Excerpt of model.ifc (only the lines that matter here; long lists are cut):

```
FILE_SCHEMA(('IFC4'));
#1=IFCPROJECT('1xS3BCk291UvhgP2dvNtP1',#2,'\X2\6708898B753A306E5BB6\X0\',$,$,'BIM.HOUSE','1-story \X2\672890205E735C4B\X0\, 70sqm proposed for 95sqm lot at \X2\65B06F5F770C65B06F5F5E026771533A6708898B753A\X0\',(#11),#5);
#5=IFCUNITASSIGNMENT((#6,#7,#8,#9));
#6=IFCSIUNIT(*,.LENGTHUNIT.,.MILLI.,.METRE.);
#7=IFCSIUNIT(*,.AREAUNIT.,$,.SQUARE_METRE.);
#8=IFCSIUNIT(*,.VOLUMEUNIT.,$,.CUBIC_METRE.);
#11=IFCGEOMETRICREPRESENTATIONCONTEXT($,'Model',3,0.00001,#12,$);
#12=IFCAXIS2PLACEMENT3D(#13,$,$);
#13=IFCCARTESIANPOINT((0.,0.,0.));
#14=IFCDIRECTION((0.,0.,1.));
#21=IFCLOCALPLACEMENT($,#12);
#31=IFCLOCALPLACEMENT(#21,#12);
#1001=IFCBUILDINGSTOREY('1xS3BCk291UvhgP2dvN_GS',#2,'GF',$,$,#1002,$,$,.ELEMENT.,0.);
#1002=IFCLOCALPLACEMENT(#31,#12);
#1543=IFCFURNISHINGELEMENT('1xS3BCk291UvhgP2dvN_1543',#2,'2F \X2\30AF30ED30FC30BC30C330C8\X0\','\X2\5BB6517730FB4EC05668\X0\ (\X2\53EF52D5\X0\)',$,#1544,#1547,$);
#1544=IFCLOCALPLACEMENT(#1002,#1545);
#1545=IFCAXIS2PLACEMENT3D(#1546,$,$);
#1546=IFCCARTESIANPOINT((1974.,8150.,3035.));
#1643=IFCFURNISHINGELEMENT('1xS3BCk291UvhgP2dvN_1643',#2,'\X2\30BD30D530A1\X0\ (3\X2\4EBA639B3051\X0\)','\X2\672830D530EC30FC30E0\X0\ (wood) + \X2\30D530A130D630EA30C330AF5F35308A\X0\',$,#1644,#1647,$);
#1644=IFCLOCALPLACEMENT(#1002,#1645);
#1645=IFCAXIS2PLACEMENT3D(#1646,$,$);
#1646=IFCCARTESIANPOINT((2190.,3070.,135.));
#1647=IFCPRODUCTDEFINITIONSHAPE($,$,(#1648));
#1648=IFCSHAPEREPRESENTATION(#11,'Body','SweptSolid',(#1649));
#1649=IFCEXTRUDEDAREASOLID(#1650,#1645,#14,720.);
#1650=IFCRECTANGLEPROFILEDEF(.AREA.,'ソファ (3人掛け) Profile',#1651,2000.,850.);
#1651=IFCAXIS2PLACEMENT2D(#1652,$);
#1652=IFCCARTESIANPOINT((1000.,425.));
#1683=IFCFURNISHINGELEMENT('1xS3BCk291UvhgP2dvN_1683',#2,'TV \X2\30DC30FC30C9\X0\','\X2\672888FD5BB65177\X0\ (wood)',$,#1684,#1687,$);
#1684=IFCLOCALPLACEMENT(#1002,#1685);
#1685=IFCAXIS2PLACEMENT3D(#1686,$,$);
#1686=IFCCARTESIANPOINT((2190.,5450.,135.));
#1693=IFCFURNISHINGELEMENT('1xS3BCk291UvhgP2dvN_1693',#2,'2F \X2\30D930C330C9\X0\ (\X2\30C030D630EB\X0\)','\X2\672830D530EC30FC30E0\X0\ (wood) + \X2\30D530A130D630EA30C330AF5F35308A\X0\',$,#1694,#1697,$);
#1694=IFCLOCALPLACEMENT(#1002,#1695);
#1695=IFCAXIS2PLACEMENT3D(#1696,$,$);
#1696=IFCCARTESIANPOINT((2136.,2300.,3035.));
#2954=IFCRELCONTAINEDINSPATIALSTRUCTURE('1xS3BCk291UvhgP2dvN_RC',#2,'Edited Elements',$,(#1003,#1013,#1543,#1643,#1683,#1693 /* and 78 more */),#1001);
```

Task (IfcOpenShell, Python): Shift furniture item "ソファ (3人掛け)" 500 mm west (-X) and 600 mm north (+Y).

```python
import ifcopenshell
import ifcopenshell.api.geometry
import ifcopenshell.util.placement

model = ifcopenshell.open("model.ifc")

item = model.by_guid("1xS3BCk291UvhgP2dvN_1643")
matrix = ifcopenshell.util.placement.get_local_placement(item.ObjectPlacement)
matrix[0, 3] -= 500.0
matrix[1, 3] += 600.0
ifcopenshell.api.geometry.edit_object_placement(model, product=item, matrix=matrix, is_si=False)

print(ifcopenshell.util.placement.get_local_placement(item.ObjectPlacement).round(3) + 0.0)

model.write("model_v2.ifc")
```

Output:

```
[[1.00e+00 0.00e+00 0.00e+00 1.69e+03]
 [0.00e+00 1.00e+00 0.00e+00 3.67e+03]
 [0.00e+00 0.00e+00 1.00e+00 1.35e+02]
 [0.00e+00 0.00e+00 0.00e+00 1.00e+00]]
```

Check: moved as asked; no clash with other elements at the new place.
